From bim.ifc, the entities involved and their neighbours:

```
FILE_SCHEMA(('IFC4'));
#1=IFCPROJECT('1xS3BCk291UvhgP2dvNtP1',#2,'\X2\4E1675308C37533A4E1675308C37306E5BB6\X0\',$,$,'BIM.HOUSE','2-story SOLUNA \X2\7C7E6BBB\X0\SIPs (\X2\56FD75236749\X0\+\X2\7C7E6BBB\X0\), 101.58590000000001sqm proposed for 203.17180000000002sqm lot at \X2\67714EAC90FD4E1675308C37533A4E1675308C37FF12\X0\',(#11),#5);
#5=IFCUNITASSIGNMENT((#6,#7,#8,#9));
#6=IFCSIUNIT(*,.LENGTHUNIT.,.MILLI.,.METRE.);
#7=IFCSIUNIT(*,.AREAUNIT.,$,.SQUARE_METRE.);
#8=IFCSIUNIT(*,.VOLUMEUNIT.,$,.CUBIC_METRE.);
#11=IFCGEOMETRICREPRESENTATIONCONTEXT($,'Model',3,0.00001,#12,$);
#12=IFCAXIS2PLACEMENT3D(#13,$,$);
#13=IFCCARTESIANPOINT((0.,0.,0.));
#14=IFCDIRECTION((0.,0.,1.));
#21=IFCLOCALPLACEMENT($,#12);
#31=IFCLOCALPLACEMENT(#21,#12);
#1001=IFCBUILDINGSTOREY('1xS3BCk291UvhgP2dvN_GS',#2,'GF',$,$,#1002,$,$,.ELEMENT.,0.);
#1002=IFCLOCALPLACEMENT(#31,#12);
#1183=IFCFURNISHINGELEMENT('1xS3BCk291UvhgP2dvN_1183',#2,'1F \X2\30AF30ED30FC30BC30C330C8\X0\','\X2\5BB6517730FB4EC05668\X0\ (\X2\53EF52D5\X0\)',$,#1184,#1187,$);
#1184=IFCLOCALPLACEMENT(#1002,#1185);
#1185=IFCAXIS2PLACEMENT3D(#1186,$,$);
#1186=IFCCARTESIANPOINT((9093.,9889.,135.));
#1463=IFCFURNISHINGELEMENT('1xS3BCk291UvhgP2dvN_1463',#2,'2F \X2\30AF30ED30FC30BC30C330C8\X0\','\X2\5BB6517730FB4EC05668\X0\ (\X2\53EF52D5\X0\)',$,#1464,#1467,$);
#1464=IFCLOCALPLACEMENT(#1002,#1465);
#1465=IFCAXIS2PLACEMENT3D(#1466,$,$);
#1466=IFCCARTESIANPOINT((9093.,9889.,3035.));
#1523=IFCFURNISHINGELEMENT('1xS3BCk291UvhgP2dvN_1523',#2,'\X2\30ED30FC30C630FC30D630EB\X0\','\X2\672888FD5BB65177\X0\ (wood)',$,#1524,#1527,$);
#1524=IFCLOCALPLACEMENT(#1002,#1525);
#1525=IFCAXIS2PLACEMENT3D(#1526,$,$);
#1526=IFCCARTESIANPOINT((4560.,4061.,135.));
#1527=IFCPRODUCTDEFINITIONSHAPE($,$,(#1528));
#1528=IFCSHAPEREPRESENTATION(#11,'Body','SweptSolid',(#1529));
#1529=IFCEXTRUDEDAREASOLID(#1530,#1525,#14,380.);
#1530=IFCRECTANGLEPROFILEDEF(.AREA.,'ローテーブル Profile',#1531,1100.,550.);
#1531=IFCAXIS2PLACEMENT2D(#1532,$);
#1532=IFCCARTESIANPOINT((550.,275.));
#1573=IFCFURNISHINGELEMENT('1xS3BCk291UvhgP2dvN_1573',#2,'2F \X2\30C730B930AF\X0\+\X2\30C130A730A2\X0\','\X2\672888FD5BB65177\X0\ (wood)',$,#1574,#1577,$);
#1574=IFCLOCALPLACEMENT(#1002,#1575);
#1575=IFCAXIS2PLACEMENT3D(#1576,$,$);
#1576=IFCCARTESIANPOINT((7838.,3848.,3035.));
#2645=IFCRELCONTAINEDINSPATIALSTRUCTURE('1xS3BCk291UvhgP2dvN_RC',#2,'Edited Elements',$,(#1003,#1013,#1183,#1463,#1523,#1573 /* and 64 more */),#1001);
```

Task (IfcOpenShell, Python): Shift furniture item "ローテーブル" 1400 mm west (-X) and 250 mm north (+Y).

```python
import ifcopenshell
import ifcopenshell.api.geometry
import ifcopenshell.util.placement
import ifcopenshell.util.unit

model = ifcopenshell.open("bim.ifc")
unit_scale = ifcopenshell.util.unit.calculate_unit_scale(model)

item = model.by_id(1523)
matrix = ifcopenshell.util.placement.get_local_placement(item.ObjectPlacement)
matrix[0, 3] -= 1.4 / unit_scale
matrix[1, 3] += 0.25 / unit_scale
ifcopenshell.api.geometry.edit_object_placement(model, product=item, matrix=matrix, is_si=False)

print(ifcopenshell.util.placement.get_local_placement(item.ObjectPlacement).round(3) + 0.0)

model.write("bim_rev.ifc")
```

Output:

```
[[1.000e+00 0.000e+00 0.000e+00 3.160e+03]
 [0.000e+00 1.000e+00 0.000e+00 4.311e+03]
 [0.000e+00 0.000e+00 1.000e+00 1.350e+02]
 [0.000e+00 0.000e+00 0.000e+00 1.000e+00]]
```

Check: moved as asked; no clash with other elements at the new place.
